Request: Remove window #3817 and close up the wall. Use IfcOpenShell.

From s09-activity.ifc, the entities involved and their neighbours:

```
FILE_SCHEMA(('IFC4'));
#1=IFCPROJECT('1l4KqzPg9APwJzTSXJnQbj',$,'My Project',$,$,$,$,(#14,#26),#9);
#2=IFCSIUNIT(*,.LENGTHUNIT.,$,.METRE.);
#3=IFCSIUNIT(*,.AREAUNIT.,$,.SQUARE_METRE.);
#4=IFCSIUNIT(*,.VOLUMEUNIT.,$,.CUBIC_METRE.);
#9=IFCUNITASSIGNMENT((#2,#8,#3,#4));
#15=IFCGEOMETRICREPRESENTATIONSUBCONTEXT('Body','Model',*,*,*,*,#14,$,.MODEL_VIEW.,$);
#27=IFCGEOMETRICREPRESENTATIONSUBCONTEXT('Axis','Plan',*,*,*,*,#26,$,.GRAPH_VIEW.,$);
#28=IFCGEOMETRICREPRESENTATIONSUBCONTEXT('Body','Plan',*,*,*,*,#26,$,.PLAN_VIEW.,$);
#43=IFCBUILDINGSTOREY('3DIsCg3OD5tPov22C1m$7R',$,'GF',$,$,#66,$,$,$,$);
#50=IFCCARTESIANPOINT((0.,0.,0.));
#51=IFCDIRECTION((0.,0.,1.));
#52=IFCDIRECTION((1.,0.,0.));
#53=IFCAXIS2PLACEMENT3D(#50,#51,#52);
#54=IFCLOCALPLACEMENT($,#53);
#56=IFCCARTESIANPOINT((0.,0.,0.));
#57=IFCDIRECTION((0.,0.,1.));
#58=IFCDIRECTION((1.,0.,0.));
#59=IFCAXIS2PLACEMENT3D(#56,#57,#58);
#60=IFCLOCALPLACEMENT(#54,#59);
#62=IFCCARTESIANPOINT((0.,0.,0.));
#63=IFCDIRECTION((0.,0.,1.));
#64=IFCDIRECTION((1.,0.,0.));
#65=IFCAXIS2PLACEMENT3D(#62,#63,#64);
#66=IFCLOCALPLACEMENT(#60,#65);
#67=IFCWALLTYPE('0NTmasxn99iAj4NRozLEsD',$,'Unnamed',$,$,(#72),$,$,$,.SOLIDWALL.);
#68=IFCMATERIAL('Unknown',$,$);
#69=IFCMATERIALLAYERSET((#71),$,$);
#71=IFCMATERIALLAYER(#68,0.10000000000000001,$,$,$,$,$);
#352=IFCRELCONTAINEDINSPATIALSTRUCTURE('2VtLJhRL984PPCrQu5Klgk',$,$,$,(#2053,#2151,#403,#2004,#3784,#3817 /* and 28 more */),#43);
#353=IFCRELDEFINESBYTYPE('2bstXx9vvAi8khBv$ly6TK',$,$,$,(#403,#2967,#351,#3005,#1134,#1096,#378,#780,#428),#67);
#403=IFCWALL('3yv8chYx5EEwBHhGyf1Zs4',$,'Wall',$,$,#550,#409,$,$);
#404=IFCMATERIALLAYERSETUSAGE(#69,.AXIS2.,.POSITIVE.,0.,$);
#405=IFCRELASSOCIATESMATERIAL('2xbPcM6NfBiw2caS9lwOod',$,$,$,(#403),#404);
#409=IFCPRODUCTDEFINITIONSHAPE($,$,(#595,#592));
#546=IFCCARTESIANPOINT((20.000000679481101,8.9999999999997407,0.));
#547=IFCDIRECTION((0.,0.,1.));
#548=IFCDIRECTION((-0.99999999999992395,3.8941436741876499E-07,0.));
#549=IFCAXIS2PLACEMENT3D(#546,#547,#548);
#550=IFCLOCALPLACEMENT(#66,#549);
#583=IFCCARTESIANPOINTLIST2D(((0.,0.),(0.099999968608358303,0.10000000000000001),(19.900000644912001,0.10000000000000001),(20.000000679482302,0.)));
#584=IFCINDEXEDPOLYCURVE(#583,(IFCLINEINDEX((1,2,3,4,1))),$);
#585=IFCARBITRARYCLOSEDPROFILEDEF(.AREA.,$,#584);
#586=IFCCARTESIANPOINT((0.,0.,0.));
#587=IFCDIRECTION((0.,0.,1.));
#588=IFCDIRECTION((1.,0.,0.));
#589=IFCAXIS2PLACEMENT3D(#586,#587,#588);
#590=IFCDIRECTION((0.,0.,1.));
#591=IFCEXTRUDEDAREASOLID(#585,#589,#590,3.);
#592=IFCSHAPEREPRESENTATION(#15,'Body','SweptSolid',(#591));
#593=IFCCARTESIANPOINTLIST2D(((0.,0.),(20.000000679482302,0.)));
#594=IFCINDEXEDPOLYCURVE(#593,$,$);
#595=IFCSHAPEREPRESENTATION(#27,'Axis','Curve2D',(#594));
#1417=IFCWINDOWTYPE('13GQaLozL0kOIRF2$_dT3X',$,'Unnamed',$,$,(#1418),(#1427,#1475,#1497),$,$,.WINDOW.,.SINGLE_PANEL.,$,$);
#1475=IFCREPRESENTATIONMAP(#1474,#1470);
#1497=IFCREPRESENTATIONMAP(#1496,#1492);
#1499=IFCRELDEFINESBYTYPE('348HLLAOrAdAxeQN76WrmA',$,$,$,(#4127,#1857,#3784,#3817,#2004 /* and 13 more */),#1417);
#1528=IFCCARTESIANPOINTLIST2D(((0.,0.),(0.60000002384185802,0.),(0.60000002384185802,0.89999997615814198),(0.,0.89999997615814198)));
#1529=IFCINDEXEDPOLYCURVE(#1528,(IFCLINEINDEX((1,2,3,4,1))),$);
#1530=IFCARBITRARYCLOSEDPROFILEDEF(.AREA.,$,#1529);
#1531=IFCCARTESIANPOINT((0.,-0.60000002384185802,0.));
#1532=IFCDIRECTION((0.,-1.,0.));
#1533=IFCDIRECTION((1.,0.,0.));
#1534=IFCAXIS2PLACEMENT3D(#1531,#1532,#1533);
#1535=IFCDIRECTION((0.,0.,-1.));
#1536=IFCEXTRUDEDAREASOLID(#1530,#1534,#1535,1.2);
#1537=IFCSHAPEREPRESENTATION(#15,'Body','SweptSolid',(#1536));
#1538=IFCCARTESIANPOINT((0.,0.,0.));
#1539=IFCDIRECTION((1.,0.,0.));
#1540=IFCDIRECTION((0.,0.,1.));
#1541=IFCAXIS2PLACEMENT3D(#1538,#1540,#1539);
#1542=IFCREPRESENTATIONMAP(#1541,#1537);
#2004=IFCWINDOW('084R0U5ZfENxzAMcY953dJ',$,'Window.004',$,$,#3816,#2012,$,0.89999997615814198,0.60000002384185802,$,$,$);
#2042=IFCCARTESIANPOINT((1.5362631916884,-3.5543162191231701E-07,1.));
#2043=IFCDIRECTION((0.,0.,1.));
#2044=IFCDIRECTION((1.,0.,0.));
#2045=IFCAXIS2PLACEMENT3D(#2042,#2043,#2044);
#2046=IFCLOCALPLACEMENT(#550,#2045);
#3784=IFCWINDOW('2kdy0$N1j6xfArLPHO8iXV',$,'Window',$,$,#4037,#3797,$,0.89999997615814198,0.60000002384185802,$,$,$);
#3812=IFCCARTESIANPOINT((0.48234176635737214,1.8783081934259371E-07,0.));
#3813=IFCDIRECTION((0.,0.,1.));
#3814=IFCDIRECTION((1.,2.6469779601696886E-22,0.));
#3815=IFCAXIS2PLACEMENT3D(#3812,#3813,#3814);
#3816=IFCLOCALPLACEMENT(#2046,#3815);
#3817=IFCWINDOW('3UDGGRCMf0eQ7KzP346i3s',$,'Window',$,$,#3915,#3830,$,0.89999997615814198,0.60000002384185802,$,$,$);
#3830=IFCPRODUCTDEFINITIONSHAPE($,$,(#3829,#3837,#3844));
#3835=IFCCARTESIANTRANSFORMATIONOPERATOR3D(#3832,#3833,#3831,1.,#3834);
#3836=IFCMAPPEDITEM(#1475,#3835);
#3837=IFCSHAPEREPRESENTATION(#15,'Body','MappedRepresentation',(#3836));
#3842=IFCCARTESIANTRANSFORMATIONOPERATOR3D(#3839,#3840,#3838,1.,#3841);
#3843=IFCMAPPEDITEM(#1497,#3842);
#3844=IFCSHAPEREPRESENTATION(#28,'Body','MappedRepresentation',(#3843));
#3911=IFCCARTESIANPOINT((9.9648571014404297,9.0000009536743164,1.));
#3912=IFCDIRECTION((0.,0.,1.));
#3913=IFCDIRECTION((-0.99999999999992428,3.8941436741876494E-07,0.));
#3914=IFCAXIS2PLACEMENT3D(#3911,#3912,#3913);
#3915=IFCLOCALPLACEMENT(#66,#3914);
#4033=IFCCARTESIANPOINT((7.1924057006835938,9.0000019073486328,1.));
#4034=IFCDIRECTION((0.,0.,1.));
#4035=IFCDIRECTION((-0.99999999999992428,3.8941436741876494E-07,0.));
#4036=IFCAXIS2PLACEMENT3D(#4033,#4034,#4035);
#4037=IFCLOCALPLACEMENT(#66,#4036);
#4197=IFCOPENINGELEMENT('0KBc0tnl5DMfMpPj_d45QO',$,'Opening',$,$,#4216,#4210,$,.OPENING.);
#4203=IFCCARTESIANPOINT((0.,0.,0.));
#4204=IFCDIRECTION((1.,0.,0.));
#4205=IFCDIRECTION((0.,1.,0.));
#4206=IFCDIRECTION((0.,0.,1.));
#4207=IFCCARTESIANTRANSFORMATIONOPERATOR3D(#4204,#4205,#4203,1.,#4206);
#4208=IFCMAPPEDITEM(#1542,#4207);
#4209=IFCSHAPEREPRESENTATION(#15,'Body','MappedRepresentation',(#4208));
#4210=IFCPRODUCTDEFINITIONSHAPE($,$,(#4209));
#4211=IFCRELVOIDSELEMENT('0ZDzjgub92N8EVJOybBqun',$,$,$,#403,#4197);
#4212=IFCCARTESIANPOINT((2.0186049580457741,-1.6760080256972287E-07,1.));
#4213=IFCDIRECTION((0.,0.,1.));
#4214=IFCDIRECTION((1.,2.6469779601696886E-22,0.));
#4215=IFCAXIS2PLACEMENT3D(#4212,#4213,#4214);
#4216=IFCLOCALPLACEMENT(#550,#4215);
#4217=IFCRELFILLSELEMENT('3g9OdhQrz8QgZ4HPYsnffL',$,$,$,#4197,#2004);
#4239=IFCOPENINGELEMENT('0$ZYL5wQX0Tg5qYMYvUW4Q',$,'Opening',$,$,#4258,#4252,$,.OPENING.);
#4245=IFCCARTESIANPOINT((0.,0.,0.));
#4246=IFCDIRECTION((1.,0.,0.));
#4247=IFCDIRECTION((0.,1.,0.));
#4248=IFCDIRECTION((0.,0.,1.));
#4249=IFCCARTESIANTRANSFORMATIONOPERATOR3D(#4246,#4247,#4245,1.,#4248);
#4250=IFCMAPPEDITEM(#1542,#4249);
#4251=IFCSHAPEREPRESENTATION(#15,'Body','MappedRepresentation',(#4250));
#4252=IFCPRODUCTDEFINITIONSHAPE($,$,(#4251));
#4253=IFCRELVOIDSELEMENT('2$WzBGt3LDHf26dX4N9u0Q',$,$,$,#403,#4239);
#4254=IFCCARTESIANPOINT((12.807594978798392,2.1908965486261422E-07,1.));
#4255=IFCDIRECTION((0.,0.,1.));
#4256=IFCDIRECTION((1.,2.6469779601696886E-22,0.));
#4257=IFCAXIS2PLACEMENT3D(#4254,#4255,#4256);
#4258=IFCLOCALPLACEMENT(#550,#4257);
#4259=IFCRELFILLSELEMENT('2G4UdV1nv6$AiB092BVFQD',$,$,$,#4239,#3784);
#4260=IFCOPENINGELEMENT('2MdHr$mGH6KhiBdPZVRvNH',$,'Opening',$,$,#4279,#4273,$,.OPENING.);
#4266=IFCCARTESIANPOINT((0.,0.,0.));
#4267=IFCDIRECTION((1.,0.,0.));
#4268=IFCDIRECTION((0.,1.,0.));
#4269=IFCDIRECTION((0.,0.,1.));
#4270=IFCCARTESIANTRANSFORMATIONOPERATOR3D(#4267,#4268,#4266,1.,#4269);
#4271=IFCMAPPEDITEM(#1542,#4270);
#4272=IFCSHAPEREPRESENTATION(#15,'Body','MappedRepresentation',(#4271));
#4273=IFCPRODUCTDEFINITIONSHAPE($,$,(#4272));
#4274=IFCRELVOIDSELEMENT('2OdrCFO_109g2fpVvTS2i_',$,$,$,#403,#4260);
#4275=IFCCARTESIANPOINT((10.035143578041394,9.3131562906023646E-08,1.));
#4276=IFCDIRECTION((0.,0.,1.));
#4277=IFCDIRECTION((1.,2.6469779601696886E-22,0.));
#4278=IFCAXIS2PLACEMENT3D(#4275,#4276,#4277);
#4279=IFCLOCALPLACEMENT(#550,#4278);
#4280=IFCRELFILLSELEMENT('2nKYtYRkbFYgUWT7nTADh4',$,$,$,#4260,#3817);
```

```python
import ifcopenshell
import ifcopenshell.api.feature
import ifcopenshell.api.root
import ifcopenshell.geom
import ifcopenshell.util.shape

model = ifcopenshell.open("s09-activity.ifc")
settings = ifcopenshell.geom.settings()


def volume(element):
    """Net volume in cubic metres, openings subtracted."""
    shape = ifcopenshell.geom.create_shape(settings, element)
    return ifcopenshell.util.shape.get_volume(shape.geometry)


window = model.by_id(3817)
opening = window.FillsVoids[0].RelatingOpeningElement
wall = opening.VoidsElements[0].RelatingBuildingElement
before = volume(wall)

ifcopenshell.api.root.remove_product(model, product=window)
ifcopenshell.api.feature.remove_feature(model, feature=opening)

after = volume(wall)

print(f"wall volume {before:.3f} -> {after:.3f} m3")

model.write("s09-activity_v2.ifc")
```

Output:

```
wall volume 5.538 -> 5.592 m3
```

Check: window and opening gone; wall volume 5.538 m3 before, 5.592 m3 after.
